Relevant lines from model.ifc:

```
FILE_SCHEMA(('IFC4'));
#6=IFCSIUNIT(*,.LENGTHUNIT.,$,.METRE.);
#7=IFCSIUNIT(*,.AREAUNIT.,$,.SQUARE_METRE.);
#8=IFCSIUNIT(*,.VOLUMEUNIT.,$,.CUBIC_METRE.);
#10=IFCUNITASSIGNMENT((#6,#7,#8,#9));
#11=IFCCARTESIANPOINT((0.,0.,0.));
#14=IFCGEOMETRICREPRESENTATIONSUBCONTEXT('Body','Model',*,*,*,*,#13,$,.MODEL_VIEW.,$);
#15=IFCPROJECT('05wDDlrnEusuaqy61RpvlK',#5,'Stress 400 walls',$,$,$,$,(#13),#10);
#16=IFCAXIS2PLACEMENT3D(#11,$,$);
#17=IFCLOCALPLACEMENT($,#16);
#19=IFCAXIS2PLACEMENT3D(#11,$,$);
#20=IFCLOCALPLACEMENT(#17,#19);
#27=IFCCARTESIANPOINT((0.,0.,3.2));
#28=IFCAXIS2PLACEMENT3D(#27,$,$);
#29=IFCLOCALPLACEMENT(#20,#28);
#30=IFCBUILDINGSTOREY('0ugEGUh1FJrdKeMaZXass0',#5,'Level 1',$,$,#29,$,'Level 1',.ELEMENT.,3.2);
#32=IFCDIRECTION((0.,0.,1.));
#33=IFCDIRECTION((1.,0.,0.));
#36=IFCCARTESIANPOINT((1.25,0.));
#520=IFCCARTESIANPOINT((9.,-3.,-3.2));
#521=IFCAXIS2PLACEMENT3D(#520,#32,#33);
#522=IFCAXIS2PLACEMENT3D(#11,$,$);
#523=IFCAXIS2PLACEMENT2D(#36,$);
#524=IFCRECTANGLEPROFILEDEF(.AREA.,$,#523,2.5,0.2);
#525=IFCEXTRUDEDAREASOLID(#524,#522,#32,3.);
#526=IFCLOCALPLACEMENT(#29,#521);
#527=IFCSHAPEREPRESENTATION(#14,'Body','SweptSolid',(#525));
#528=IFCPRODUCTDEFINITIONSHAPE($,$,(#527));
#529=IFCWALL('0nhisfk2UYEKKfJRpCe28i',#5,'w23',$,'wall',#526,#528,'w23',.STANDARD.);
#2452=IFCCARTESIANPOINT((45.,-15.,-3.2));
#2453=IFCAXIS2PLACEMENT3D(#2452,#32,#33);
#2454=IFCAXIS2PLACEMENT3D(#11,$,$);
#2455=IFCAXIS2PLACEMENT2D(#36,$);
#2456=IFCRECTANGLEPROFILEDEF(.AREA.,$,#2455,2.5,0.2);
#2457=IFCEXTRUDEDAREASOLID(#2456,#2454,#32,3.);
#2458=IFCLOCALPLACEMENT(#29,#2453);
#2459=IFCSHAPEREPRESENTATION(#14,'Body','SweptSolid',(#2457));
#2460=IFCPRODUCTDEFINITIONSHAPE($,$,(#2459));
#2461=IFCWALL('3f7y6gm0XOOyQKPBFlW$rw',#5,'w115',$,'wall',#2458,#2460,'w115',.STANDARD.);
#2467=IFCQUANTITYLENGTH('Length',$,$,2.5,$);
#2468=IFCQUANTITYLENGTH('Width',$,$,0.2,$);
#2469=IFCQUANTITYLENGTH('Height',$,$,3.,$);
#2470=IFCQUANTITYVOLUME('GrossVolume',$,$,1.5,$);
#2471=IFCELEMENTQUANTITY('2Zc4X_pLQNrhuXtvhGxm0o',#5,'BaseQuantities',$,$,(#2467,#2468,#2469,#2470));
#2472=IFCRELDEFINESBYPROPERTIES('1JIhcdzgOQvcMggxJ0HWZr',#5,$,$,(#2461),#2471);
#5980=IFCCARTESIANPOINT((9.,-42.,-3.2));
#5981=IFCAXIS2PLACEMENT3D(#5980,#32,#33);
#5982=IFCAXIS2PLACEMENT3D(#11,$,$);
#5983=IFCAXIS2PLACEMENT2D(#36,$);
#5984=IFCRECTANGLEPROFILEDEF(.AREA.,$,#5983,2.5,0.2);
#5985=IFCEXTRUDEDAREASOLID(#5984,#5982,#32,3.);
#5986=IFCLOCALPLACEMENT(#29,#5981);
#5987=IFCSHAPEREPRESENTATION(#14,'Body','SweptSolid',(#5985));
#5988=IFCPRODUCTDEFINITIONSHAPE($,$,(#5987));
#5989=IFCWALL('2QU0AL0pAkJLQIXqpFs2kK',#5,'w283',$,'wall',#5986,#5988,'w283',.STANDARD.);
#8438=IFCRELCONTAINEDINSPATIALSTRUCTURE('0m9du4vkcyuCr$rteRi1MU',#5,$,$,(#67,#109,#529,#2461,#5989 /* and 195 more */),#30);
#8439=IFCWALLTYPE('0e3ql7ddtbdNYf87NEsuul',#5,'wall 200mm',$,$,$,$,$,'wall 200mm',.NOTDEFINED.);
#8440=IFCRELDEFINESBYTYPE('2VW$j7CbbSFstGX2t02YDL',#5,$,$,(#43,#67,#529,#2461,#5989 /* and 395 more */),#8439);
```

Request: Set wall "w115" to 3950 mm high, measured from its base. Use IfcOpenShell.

```python
import ifcopenshell
import ifcopenshell.api.pset
import ifcopenshell.geom
import ifcopenshell.util.element
import ifcopenshell.util.representation
import ifcopenshell.util.shape
import ifcopenshell.util.unit

model = ifcopenshell.open("model.ifc")
unit_scale = ifcopenshell.util.unit.calculate_unit_scale(model)
volume_scale = ifcopenshell.util.unit.calculate_unit_scale(model, "VOLUMEUNIT")
settings = ifcopenshell.geom.settings()


def volume(element):
    """Net volume in cubic metres, openings subtracted."""
    shape = ifcopenshell.geom.create_shape(settings, element)
    return ifcopenshell.util.shape.get_volume(shape.geometry)


wall = model.by_id(2461)
before = volume(wall)

body = ifcopenshell.util.representation.get_representation(wall, "Model", "Body")
solid = body.Items[0]
old_height = solid.Depth
solid.Depth = 3.95 / unit_scale
after = volume(wall)

# Update the stored height, areas and volumes.
qto = model.by_id(ifcopenshell.util.element.get_pset(wall, "BaseQuantities", should_inherit=False)["id"])
ifcopenshell.api.pset.edit_qto(model, qto=qto, properties={
    "Height": solid.Depth,
    "GrossVolume": ifcopenshell.util.element.get_pset(wall, "BaseQuantities", "GrossVolume") * solid.Depth / old_height,
})

print(f"height {old_height:g} -> {solid.Depth:g}, volume {before:.3f} -> {after:.3f} m3")

model.write("model_v2.ifc")
```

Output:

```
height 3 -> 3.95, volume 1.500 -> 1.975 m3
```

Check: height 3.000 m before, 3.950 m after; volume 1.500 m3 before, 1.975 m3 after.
